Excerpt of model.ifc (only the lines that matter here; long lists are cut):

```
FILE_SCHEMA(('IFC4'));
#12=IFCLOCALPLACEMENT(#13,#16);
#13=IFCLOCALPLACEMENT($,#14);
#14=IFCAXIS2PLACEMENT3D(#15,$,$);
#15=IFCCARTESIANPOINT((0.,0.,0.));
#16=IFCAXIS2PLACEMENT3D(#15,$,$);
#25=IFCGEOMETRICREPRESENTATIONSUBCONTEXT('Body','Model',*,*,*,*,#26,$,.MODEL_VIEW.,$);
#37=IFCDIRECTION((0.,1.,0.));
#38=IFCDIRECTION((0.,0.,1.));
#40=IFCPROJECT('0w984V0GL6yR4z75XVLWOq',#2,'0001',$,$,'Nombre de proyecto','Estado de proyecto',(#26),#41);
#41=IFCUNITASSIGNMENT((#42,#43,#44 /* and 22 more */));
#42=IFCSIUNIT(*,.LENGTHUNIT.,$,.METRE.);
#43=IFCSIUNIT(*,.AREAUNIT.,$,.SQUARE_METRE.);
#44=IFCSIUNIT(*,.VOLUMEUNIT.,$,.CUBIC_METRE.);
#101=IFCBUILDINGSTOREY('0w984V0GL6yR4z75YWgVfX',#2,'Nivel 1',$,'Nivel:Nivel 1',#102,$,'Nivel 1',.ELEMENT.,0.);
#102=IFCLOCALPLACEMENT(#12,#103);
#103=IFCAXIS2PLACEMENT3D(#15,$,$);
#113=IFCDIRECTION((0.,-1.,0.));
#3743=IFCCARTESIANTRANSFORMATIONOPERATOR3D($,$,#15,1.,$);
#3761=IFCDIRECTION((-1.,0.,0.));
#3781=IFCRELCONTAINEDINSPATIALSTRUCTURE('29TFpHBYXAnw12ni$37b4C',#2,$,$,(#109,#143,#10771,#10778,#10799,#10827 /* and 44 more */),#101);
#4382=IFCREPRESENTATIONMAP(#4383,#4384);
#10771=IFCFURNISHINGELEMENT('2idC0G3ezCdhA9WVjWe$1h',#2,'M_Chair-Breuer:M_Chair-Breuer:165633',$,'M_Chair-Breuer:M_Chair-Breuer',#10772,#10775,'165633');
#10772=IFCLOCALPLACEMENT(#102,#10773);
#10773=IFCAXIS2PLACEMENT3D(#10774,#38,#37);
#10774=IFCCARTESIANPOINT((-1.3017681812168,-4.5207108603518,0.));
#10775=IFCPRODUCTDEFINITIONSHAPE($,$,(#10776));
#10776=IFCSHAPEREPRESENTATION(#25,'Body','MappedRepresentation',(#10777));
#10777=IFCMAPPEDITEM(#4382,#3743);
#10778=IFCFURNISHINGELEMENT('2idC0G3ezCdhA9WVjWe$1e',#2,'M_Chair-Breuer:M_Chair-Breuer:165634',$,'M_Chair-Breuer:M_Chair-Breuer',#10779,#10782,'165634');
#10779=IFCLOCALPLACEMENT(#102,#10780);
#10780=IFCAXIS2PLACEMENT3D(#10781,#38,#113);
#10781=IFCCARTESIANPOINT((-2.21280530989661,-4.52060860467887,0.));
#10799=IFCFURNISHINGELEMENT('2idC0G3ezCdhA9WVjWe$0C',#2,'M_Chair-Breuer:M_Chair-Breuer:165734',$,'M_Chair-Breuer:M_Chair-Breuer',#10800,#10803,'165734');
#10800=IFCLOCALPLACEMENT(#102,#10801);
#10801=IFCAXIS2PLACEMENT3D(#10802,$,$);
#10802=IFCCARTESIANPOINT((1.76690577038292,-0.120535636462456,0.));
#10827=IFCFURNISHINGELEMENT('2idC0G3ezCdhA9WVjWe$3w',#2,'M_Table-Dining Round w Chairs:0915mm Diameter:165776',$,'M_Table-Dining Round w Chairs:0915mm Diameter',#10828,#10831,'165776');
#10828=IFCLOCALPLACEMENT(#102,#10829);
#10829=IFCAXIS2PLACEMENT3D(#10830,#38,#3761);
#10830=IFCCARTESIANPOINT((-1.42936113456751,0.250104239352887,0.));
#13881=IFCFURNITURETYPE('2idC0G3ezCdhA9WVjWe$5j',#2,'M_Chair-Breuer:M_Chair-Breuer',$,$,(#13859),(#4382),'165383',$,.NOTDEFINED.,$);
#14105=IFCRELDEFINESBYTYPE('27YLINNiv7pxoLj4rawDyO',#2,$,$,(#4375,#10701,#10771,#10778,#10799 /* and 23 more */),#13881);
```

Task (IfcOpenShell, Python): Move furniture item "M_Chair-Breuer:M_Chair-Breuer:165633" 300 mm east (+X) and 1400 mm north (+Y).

```python
import ifcopenshell
import ifcopenshell.api.geometry
import ifcopenshell.util.placement
import ifcopenshell.util.unit

model = ifcopenshell.open("model.ifc")
unit_scale = ifcopenshell.util.unit.calculate_unit_scale(model)

item = model.by_id(10771)
matrix = ifcopenshell.util.placement.get_local_placement(item.ObjectPlacement)
matrix[0, 3] += 0.3 / unit_scale
matrix[1, 3] += 1.4 / unit_scale
ifcopenshell.api.geometry.edit_object_placement(model, product=item, matrix=matrix, is_si=False)

print(ifcopenshell.util.placement.get_local_placement(item.ObjectPlacement).round(3) + 0.0)

model.write("model_edited.ifc")
```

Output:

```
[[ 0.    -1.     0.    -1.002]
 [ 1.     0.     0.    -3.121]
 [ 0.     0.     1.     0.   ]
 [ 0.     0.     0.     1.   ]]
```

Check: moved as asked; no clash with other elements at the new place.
